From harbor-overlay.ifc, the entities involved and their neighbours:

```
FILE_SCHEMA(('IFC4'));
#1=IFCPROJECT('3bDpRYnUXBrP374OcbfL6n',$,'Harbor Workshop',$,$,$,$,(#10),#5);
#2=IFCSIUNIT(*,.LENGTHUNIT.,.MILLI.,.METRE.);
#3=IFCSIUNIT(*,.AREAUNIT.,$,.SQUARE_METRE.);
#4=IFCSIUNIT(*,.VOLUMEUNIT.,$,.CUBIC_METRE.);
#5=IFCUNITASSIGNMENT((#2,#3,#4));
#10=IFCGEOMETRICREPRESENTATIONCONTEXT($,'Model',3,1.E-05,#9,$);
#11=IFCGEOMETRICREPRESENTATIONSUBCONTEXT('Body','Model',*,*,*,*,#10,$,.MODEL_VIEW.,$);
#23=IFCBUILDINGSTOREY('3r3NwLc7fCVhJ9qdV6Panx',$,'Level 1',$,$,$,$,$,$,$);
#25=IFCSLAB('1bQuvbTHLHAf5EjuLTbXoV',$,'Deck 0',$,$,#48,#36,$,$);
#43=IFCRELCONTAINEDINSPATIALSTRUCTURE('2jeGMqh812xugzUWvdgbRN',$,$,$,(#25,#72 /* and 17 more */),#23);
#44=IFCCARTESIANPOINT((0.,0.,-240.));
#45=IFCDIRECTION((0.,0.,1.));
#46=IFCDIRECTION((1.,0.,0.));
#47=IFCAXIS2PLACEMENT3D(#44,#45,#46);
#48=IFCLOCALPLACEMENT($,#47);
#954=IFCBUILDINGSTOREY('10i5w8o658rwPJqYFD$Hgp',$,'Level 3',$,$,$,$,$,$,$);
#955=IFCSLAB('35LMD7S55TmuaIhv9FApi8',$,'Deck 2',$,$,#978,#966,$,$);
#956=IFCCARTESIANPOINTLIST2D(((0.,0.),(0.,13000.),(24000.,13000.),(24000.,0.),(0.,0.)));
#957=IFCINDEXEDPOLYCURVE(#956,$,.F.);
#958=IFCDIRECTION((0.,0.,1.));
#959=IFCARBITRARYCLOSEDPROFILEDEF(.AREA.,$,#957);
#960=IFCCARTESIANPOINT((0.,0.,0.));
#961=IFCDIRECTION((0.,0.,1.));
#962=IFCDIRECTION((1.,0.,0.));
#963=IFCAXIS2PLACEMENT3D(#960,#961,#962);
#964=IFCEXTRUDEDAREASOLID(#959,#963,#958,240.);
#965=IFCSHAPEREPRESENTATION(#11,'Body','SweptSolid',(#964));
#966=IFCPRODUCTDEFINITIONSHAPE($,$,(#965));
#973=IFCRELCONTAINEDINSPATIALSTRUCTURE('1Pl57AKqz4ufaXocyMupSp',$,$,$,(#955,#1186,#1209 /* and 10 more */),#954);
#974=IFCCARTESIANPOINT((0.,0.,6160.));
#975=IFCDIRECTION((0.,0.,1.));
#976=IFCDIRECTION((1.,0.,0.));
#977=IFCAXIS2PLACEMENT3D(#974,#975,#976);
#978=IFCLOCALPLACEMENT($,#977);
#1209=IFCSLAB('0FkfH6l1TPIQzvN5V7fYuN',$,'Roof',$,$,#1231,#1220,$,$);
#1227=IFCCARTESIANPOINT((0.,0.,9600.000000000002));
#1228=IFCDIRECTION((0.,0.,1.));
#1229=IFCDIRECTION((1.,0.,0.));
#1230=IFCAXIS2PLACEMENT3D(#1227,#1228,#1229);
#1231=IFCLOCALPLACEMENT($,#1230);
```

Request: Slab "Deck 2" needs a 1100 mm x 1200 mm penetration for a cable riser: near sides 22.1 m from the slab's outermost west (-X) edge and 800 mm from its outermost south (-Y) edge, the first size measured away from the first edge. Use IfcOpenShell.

```python
import numpy as np
import ifcopenshell
import ifcopenshell.api.feature
import ifcopenshell.api.geometry
import ifcopenshell.api.root
import ifcopenshell.geom
import ifcopenshell.util.placement
import ifcopenshell.util.representation
import ifcopenshell.util.shape
import ifcopenshell.util.unit

model = ifcopenshell.open("harbor-overlay.ifc")
unit_scale = ifcopenshell.util.unit.calculate_unit_scale(model)
settings = ifcopenshell.geom.settings()


def volume(element):
    """Net volume in cubic metres, openings subtracted."""
    shape = ifcopenshell.geom.create_shape(settings, element)
    return ifcopenshell.util.shape.get_volume(shape.geometry)


slab = model.by_guid("35LMD7S55TmuaIhv9FApi8")
before = volume(slab)

# Extent in the slab's own axes, in metres. The edges named are its -X and -Y sides.
slab_shape = ifcopenshell.geom.create_shape(settings, slab)
vertices = ifcopenshell.util.shape.get_vertices(slab_shape.geometry)
x_min, y_min, bottom = vertices.min(axis=0)
top = vertices[:, 2].max()

opening = ifcopenshell.api.root.create_entity(model, ifc_class="IfcOpeningElement", name="Cable riser opening", predefined_type="OPENING")
context = ifcopenshell.util.representation.get_context(model, "Model", "Body", "MODEL_VIEW")
width, depth = 1.1, 1.2
outline = [(0.0, 0.0), (width, 0.0), (width, depth), (0.0, depth), (0.0, 0.0)]
# Overshoot both faces by 50 mm so the cut is clean.
shape = ifcopenshell.api.geometry.add_slab_representation(
    model, context=context, depth=top - bottom + 0.1, polyline=outline
)
ifcopenshell.api.geometry.assign_representation(model, product=opening, representation=shape)

matrix = ifcopenshell.util.placement.get_local_placement(slab.ObjectPlacement)
matrix[:, 3] = matrix @ np.append(np.array([x_min + 22.1, y_min + 0.8, bottom - 0.05]) / unit_scale, 1.0)
ifcopenshell.api.geometry.edit_object_placement(model, product=opening, matrix=matrix, is_si=False)
ifcopenshell.api.feature.add_feature(model, feature=opening, element=slab)

after = volume(slab)

print(f"slab volume {before:.3f} -> {after:.3f} m3")

model.write("harbor-overlay-out.ifc")
```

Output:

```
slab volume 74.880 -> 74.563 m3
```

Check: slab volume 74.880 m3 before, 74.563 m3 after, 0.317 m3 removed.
